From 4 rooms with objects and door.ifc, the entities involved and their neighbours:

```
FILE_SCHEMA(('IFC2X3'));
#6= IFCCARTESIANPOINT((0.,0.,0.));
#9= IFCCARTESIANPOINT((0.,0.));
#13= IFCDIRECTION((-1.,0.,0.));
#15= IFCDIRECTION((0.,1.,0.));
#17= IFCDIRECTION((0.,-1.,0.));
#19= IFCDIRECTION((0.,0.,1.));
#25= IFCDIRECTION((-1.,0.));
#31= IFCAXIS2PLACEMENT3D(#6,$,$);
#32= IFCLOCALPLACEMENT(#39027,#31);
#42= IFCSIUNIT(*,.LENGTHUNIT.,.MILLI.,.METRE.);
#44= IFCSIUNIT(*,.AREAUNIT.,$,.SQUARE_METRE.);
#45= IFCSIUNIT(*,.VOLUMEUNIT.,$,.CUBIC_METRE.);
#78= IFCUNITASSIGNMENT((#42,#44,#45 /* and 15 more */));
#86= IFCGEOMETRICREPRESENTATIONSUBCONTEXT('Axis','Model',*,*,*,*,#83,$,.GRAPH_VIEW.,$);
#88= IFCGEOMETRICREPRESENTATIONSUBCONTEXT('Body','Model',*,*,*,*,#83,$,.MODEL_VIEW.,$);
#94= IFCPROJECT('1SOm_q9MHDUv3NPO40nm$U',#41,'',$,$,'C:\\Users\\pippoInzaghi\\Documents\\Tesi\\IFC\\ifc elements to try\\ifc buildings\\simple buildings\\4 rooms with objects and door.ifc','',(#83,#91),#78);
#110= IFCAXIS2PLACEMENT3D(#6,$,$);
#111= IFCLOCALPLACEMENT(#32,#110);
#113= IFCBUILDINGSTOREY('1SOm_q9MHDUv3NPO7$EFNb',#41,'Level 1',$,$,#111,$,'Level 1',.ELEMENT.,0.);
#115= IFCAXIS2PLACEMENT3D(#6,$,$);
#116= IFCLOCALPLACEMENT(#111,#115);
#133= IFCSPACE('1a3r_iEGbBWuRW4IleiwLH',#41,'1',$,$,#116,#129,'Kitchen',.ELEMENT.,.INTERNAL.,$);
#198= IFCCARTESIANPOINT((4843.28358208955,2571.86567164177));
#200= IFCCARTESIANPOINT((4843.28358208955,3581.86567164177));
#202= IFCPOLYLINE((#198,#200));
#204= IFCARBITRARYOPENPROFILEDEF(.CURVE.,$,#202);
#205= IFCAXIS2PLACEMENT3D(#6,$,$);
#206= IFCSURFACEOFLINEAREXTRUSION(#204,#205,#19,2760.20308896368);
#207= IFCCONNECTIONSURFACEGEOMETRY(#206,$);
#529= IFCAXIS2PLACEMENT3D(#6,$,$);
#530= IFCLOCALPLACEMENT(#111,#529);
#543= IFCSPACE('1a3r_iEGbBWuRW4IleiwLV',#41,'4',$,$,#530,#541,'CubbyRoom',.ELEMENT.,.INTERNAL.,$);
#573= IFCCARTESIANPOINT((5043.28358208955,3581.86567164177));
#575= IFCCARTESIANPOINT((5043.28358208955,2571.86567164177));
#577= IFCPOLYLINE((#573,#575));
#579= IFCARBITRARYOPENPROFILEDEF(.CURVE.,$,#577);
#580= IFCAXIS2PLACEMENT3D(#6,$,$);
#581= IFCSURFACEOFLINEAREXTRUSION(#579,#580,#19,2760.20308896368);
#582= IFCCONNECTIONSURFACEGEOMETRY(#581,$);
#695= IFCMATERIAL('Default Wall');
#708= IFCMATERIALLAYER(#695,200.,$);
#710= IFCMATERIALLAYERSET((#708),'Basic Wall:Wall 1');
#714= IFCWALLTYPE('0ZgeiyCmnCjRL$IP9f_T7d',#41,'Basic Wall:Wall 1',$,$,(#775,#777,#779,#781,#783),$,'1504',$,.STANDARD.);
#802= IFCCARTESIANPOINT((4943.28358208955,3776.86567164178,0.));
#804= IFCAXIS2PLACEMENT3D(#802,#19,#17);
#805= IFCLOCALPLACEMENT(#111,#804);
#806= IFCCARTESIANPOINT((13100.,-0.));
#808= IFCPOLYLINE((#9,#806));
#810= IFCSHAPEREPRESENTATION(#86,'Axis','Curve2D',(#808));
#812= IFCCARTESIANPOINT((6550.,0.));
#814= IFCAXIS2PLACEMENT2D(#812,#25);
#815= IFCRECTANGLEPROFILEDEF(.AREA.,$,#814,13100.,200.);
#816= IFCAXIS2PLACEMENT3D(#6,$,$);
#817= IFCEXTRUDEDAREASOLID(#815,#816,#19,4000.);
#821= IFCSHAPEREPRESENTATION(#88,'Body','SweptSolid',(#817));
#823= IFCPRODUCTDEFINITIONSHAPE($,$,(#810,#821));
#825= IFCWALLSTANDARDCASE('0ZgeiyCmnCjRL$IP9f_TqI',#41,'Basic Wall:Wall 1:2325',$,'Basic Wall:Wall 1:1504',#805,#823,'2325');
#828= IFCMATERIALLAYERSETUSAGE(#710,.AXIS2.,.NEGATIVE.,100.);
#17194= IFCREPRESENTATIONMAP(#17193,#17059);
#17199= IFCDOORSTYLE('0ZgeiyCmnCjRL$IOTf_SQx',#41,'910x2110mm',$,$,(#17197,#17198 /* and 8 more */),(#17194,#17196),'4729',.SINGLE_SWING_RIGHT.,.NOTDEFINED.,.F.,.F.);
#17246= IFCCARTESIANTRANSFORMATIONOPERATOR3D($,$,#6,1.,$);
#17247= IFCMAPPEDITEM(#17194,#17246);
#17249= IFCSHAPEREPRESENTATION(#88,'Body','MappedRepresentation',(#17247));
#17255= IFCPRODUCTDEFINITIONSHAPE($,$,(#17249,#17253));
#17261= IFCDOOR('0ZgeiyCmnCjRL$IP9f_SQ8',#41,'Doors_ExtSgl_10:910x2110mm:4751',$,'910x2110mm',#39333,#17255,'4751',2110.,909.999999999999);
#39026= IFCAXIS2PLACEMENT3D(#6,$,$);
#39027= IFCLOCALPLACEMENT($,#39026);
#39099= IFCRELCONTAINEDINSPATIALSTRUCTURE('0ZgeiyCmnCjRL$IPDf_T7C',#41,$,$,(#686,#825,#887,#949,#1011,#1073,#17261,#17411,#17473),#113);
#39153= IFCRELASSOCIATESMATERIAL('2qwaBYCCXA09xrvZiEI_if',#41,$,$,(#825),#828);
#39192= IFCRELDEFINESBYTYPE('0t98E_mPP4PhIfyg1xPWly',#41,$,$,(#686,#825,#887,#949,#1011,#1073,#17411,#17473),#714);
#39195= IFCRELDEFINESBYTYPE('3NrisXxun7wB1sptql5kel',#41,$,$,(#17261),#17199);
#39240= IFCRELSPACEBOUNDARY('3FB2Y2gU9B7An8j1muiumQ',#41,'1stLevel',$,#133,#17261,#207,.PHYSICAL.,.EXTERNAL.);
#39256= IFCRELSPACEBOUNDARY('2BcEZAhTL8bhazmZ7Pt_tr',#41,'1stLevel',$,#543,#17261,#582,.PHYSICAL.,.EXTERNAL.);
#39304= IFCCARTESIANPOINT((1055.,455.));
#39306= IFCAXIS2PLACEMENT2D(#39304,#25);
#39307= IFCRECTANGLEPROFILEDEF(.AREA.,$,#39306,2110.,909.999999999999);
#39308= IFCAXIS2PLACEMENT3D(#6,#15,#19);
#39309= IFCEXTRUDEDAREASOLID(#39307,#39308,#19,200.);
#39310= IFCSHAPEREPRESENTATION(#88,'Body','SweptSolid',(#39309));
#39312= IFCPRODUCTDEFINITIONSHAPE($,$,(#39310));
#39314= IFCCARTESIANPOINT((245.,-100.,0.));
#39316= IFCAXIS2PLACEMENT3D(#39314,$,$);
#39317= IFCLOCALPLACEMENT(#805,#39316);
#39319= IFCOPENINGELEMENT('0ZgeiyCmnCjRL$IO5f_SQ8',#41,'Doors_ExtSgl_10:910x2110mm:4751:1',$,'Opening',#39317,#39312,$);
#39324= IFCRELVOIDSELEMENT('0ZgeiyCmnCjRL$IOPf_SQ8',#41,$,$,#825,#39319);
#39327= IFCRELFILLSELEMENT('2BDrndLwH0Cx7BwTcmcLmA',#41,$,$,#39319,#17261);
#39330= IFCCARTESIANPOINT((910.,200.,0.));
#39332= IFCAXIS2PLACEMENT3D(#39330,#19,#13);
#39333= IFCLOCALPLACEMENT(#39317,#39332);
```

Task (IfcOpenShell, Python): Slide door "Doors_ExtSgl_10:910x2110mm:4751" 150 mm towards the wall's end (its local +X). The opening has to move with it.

```python
import numpy as np
import ifcopenshell
import ifcopenshell.api.geometry
import ifcopenshell.util.placement

model = ifcopenshell.open("4 rooms with objects and door.ifc")

door = model.by_id(17261)
opening = door.FillsVoids[0].RelatingOpeningElement
wall = opening.VoidsElements[0].RelatingBuildingElement

wall_matrix = ifcopenshell.util.placement.get_local_placement(wall.ObjectPlacement)
shift = wall_matrix[:3, 0] * 150.0
before = ifcopenshell.util.placement.get_local_placement(door.ObjectPlacement)[:3, 3].copy()

# The door is placed relative to its opening, so it follows when the opening moves.
matrix = ifcopenshell.util.placement.get_local_placement(opening.ObjectPlacement)
matrix[:3, 3] += shift
ifcopenshell.api.geometry.edit_object_placement(
    model, product=opening, matrix=matrix, is_si=False, should_transform_children=True
)

# Space boundary surfaces are stored in each space's coordinates; move them too.
for rel in door.ProvidesBoundaries:
    if not rel.ConnectionGeometry:
        continue
    surface = rel.ConnectionGeometry.SurfaceOnRelatingElement
    space_matrix = ifcopenshell.util.placement.get_local_placement(rel.RelatingSpace.ObjectPlacement)
    point = np.array(surface.Position.Location.Coordinates) + space_matrix[:3, :3].T @ shift
    surface.Position = model.createIfcAxis2Placement3D(
        model.createIfcCartesianPoint(point.tolist()), surface.Position.Axis, surface.Position.RefDirection
    )

after = ifcopenshell.util.placement.get_local_placement(door.ObjectPlacement)[:3, 3]
print("door moved by", (after - before).round(3) + 0.0)

model.write("4 rooms with objects and door-out.ifc")
```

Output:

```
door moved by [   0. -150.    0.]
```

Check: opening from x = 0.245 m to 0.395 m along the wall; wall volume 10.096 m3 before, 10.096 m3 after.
